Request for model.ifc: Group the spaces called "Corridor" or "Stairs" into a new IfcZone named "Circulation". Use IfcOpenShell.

First a look at what the model holds.

```python
import ifcopenshell

model = ifcopenshell.open("model.ifc")
print(model.schema)
seen = {}
for space in model.by_type("IfcSpace"):
    seen[space.LongName] = seen.get(space.LongName, 0) + 1
for name, count in sorted(seen.items(), key=str):
    print(count, "x", name)
print("zones:", [z.Name for z in model.by_type("IfcZone")][:20])
```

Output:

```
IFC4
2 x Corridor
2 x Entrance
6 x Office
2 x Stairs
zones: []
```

```python
import ifcopenshell
import ifcopenshell.api.group
import ifcopenshell.api.root

model = ifcopenshell.open("model.ifc")

names = {"Corridor", "Stairs"}
spaces = [s for s in model.by_type("IfcSpace") if s.LongName in names]

zone = ifcopenshell.api.root.create_entity(model, ifc_class="IfcZone", name="Circulation")
ifcopenshell.api.group.assign_group(model, products=spaces, group=zone)
print(len(spaces), "spaces in", zone.Name)

model.write("model_v2.ifc")
```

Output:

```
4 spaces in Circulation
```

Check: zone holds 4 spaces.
